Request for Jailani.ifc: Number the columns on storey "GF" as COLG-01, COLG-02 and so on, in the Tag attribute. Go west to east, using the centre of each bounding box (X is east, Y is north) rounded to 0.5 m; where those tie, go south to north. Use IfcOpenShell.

First a look at what the model holds.

```python
import ifcopenshell
import ifcopenshell.util.element
import ifcopenshell.util.placement

model = ifcopenshell.open("Jailani.ifc")
print(model.schema)
storey = next(s for s in model.by_type("IfcBuildingStorey") if s.Name == "GF")
columns = [e for e in ifcopenshell.util.element.get_decomposition(storey) if e.is_a("IfcColumn")]
for e in sorted(columns, key=lambda e: e.id()):
    origin = ifcopenshell.util.placement.get_local_placement(e.ObjectPlacement)[:3, 3]
    print(e.id(), e.Tag, e.Name, origin.round(2) + 0.0, sep=" | ")
```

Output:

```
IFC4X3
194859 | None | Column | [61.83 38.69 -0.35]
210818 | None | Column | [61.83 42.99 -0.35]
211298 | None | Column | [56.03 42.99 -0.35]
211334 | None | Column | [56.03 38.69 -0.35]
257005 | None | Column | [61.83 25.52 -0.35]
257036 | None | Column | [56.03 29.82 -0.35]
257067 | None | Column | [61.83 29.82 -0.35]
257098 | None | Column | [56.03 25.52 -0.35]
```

```python
import ifcopenshell
import ifcopenshell.geom
import ifcopenshell.util.element
import ifcopenshell.util.shape

model = ifcopenshell.open("Jailani.ifc")
settings = ifcopenshell.geom.settings()
settings.set("use-world-coords", True)


def centre(element):
    shape = ifcopenshell.geom.create_shape(settings, element)
    return ifcopenshell.util.shape.get_bbox_centroid(shape.geometry)


storey = next(s for s in model.by_type("IfcBuildingStorey") if s.Name == "GF")
columns = [e for e in ifcopenshell.util.element.get_decomposition(storey) if e.is_a("IfcColumn")]

# Insertion points can sit at a corner or the storey origin, so sort by the geometry (in metres).
centres = {e: centre(e) for e in columns}
columns.sort(key=lambda e: (round(centres[e][0] / 0.5), centres[e][1]))

for i, e in enumerate(columns, start=1):
    number = f"COLG-{i:02d}"
    e.Tag = number
    print(e.id(), number)

model.write("Jailani_v2.ifc")
```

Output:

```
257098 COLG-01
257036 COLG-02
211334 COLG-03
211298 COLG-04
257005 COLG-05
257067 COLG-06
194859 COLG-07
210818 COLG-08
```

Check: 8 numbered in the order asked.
